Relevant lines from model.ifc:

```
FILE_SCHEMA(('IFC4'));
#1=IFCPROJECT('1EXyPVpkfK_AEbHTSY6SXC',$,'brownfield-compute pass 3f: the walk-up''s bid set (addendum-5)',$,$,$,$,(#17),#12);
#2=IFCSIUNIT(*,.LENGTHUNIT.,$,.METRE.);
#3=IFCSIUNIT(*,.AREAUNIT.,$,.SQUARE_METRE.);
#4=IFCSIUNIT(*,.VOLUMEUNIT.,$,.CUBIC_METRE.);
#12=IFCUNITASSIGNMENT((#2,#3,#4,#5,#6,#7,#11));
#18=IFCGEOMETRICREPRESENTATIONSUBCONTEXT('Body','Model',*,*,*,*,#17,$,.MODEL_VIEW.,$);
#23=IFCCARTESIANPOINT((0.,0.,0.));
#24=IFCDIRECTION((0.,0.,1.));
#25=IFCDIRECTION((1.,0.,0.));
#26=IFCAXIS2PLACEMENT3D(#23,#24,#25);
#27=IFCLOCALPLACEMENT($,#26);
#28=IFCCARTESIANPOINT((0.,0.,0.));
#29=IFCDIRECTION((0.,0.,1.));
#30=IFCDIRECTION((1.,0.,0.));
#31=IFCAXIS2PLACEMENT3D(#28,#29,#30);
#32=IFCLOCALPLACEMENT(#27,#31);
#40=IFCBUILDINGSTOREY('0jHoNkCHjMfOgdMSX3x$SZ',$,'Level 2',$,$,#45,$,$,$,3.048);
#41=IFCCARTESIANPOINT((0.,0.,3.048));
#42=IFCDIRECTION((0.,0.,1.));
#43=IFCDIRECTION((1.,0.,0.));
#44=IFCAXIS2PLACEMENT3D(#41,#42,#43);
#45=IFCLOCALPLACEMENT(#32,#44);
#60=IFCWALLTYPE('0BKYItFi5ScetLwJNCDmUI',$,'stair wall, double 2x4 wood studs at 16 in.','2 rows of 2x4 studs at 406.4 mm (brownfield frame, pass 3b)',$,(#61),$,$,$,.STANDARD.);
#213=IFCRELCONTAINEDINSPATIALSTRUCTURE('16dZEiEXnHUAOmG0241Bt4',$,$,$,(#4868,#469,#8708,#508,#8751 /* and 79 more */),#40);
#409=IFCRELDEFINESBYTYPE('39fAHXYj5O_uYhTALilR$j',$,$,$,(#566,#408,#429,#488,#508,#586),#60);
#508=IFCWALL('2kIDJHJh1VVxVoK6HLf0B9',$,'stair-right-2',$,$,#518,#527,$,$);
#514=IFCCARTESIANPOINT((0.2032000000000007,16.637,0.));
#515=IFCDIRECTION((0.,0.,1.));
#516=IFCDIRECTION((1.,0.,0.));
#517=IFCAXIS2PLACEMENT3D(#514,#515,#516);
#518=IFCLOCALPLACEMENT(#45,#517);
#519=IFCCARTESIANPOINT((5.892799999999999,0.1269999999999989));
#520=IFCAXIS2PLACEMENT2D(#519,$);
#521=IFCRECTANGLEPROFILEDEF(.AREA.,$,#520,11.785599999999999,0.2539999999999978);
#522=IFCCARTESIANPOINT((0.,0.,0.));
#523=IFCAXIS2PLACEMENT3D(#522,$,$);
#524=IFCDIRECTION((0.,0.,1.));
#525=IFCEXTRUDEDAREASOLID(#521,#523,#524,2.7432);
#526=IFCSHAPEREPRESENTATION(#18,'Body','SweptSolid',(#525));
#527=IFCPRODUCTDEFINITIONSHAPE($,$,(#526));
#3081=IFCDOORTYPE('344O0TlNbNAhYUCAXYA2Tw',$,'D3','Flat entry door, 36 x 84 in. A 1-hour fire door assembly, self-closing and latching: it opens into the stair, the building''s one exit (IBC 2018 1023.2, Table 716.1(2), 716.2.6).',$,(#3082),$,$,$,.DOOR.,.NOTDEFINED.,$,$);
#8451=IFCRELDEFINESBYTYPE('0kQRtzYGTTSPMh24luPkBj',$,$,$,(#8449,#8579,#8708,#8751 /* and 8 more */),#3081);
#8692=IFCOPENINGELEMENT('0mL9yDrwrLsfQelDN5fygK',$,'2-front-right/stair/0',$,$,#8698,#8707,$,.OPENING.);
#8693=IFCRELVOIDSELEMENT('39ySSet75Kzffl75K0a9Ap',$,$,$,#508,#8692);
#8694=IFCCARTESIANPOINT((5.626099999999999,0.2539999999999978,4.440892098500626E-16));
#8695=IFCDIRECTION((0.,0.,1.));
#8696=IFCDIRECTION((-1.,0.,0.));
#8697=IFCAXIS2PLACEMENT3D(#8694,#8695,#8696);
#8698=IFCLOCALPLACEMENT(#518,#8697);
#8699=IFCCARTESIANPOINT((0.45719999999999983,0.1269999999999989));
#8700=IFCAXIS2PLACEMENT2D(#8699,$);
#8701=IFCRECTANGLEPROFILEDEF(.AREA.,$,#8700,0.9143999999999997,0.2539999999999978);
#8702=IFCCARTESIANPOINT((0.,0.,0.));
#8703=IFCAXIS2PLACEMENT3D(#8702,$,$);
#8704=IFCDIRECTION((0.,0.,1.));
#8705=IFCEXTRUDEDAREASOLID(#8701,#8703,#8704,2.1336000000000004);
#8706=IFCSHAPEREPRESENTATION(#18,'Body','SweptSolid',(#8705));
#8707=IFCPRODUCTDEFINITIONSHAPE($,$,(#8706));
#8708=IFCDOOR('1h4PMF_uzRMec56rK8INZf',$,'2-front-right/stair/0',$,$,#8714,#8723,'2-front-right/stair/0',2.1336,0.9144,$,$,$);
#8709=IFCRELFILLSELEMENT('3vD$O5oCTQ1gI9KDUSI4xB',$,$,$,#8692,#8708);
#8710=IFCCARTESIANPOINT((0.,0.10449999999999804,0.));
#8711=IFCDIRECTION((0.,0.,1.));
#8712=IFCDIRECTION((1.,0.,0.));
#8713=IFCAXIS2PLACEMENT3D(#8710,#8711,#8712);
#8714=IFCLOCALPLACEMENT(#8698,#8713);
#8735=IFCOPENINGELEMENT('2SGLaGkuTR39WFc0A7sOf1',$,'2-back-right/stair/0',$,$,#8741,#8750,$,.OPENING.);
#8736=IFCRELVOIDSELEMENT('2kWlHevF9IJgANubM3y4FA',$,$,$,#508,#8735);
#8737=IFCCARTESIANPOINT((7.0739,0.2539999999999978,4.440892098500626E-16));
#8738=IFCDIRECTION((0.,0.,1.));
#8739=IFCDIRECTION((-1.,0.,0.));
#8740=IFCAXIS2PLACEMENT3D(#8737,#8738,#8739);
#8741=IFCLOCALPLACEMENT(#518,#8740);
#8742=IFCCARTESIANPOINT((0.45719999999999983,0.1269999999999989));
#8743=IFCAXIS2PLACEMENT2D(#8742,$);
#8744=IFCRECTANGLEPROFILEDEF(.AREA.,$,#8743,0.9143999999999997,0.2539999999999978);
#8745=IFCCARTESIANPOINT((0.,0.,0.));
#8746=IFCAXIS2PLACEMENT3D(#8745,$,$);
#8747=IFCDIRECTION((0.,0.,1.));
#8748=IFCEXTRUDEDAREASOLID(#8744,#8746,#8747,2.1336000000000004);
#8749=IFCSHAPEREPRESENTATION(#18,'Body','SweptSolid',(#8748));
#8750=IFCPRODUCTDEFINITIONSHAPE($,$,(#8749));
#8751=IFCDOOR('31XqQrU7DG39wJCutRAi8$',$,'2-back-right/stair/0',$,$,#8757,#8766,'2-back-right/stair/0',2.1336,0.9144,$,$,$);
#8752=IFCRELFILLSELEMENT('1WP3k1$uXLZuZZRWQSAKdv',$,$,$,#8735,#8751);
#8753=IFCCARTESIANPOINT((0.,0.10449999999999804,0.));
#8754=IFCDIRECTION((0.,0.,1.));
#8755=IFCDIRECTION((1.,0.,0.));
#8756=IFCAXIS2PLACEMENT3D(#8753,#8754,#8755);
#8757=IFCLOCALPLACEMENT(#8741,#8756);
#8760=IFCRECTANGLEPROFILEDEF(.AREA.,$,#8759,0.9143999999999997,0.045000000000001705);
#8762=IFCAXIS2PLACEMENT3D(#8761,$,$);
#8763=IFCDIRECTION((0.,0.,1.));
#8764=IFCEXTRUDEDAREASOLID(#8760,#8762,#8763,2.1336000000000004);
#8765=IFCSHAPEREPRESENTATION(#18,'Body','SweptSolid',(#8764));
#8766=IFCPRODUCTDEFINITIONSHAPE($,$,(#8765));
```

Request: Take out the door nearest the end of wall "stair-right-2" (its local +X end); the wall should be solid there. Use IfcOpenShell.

```python
import ifcopenshell
import ifcopenshell.api.feature
import ifcopenshell.api.root
import ifcopenshell.geom
import ifcopenshell.util.shape

model = ifcopenshell.open("model.ifc")
settings = ifcopenshell.geom.settings()


def volume(element):
    """Net volume in cubic metres, openings subtracted."""
    shape = ifcopenshell.geom.create_shape(settings, element)
    return ifcopenshell.util.shape.get_volume(shape.geometry)


door = model.by_guid("31XqQrU7DG39wJCutRAi8$")
opening = door.FillsVoids[0].RelatingOpeningElement
wall = opening.VoidsElements[0].RelatingBuildingElement
before = volume(wall)

ifcopenshell.api.root.remove_product(model, product=door)
ifcopenshell.api.feature.remove_feature(model, feature=opening)

after = volume(wall)

print(f"wall volume {before:.3f} -> {after:.3f} m3")

model.write("model_rev.ifc")
```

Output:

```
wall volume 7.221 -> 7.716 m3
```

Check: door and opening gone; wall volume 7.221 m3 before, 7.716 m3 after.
